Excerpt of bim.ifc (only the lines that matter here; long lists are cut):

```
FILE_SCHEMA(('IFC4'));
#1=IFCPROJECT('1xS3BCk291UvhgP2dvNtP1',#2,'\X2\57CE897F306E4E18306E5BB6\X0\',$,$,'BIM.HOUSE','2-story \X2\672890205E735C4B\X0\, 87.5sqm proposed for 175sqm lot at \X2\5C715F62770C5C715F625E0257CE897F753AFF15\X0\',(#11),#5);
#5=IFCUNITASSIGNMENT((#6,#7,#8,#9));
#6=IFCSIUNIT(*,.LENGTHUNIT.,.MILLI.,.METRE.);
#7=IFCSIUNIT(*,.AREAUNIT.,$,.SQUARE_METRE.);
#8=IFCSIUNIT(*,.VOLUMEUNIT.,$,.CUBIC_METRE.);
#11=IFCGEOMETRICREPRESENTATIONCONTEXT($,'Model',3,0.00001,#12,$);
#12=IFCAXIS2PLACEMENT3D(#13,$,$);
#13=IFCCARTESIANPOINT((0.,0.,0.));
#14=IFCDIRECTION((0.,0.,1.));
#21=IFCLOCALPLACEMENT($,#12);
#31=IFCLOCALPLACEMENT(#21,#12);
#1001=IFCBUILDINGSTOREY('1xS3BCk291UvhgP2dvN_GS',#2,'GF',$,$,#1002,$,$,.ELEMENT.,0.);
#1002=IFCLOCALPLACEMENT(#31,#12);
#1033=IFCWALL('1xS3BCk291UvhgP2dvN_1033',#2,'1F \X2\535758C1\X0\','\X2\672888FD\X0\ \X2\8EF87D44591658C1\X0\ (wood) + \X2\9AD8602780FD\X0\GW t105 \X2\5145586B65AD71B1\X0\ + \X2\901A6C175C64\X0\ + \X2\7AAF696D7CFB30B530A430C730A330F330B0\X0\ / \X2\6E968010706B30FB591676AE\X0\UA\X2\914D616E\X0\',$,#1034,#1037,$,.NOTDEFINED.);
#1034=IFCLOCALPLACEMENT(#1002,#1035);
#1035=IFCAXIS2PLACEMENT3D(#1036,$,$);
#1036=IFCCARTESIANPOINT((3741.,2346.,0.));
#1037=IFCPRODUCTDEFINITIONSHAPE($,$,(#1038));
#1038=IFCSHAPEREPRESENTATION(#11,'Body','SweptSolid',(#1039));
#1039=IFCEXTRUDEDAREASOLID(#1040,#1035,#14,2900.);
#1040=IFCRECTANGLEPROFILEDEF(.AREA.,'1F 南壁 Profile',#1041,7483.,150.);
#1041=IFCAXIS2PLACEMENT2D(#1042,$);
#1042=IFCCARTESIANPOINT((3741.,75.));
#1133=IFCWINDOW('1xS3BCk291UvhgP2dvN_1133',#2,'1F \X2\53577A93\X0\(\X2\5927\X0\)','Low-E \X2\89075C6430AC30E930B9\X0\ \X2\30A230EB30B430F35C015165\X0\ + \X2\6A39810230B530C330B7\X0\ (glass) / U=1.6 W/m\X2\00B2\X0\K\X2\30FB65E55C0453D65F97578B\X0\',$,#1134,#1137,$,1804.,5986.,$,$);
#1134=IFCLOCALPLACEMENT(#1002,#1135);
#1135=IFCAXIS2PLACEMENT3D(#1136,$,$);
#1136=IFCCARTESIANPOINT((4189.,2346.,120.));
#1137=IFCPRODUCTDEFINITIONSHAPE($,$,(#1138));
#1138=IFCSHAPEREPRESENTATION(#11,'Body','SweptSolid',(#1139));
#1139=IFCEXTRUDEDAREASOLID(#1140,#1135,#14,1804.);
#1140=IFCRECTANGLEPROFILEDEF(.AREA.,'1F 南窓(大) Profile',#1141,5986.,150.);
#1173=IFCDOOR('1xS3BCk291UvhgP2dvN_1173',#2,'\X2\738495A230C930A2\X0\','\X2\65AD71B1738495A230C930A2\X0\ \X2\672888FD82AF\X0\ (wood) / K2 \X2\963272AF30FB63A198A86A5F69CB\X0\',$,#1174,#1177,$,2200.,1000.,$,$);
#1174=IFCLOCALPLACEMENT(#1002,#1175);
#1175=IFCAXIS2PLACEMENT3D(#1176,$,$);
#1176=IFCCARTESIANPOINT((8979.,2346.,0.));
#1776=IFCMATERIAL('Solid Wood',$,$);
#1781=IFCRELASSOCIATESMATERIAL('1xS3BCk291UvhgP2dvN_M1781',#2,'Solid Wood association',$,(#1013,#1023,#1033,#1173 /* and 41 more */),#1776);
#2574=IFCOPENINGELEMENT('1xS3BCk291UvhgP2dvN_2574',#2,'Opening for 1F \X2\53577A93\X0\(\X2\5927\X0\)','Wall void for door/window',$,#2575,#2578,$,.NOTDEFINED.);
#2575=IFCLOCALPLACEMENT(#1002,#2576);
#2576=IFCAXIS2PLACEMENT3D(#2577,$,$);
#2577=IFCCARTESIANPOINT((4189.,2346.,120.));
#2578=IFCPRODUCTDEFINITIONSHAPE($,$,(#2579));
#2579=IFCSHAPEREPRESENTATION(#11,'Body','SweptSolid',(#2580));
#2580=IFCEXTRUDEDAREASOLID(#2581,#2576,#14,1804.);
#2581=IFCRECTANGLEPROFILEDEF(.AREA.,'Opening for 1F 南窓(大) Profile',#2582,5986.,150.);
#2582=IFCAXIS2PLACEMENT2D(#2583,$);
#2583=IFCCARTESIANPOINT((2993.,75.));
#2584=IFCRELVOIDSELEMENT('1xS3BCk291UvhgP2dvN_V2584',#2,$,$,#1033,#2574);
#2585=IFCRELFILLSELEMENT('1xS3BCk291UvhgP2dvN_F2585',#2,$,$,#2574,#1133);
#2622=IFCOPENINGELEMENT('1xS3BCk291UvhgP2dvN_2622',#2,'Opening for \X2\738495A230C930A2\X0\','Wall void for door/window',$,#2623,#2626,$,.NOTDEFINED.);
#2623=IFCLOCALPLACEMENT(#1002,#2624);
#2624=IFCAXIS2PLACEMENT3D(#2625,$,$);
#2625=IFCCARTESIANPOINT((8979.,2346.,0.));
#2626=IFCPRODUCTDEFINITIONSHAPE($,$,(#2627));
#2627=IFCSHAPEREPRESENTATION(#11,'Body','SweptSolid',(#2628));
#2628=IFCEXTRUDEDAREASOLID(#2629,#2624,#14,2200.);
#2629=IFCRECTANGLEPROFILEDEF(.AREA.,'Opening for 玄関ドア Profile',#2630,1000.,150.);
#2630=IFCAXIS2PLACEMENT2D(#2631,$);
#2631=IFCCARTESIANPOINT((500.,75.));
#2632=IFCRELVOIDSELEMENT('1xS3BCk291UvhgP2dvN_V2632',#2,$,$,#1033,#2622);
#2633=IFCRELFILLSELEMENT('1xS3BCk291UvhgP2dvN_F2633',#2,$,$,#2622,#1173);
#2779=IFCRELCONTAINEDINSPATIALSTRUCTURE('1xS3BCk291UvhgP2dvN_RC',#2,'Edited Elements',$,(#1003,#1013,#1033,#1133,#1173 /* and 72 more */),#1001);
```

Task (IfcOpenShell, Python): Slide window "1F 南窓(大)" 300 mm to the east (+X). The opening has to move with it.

```python
import ifcopenshell
import ifcopenshell.api.geometry
import ifcopenshell.util.placement
import ifcopenshell.util.unit

model = ifcopenshell.open("bim.ifc")
unit_scale = ifcopenshell.util.unit.calculate_unit_scale(model)

window = model.by_guid("1xS3BCk291UvhgP2dvN_1133")
opening = window.FillsVoids[0].RelatingOpeningElement
wall = opening.VoidsElements[0].RelatingBuildingElement

wall_matrix = ifcopenshell.util.placement.get_local_placement(wall.ObjectPlacement)
shift = wall_matrix[:3, 0] * 0.3 / unit_scale
before = ifcopenshell.util.placement.get_local_placement(window.ObjectPlacement)[:3, 3].copy()

# The window is not placed relative to its opening, so move both.
for product in (opening, window):
    matrix = ifcopenshell.util.placement.get_local_placement(product.ObjectPlacement)
    matrix[:3, 3] += shift
    ifcopenshell.api.geometry.edit_object_placement(model, product=product, matrix=matrix, is_si=False)

after = ifcopenshell.util.placement.get_local_placement(window.ObjectPlacement)[:3, 3]
print("window moved by", (after - before).round(3) + 0.0)

model.write("bim_v2.ifc")
```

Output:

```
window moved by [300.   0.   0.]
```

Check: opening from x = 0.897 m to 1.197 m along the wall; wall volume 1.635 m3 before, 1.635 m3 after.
